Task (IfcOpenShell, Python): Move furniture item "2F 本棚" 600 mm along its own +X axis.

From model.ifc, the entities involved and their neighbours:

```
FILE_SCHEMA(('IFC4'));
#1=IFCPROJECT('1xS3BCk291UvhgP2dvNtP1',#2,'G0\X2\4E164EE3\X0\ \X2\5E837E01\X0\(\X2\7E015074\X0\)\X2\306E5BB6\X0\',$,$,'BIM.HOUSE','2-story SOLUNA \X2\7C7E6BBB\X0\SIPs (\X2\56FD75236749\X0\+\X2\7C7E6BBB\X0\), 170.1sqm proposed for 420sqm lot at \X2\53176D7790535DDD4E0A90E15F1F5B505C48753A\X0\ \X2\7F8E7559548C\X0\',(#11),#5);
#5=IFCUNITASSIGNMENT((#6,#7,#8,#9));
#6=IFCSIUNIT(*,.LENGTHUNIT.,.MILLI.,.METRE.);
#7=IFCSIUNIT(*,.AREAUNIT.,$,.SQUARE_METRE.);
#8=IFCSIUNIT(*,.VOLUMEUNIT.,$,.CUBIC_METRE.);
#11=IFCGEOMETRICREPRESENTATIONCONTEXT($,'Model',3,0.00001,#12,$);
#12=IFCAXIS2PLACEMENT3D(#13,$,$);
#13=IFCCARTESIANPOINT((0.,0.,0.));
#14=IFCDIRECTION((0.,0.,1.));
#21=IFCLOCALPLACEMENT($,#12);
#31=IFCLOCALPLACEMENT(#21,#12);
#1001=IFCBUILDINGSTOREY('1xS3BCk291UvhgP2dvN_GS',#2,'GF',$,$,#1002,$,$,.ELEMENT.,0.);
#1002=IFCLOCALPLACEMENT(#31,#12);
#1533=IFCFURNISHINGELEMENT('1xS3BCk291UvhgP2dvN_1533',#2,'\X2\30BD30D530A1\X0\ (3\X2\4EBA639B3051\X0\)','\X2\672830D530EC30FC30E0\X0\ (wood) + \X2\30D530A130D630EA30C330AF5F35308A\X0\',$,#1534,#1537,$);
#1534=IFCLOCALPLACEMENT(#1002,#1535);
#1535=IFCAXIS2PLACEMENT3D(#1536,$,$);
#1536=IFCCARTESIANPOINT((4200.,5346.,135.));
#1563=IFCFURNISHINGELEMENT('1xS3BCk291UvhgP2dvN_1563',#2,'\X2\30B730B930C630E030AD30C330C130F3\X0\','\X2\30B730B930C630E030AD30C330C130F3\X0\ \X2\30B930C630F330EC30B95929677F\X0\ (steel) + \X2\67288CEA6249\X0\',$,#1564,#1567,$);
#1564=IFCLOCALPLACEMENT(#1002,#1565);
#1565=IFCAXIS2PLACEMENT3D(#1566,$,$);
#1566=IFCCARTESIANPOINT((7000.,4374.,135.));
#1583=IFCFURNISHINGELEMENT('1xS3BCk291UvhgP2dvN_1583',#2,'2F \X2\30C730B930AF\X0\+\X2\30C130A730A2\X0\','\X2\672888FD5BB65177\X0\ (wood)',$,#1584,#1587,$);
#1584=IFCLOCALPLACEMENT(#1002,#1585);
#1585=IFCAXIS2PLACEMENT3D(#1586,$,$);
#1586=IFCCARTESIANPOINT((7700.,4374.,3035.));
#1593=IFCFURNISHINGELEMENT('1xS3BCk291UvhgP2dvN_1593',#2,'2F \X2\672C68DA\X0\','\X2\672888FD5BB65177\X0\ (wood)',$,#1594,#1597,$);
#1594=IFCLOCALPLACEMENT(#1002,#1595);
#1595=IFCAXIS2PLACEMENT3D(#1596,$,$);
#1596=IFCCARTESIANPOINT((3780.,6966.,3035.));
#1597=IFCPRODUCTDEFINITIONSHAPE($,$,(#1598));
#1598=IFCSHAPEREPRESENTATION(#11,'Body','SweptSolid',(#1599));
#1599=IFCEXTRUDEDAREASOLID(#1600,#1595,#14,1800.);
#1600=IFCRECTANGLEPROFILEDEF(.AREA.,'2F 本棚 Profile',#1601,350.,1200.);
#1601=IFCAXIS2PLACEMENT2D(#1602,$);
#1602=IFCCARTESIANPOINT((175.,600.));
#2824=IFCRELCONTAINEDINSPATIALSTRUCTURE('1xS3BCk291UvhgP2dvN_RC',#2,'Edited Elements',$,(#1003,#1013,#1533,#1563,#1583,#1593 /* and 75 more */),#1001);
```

```python
import ifcopenshell
import ifcopenshell.api.geometry
import ifcopenshell.util.placement
import ifcopenshell.util.unit

model = ifcopenshell.open("model.ifc")
unit_scale = ifcopenshell.util.unit.calculate_unit_scale(model)

item = model.by_id(1593)
matrix = ifcopenshell.util.placement.get_local_placement(item.ObjectPlacement)
matrix[:3, 3] += matrix[:3, 0] * 0.6 / unit_scale
ifcopenshell.api.geometry.edit_object_placement(model, product=item, matrix=matrix, is_si=False)

print(ifcopenshell.util.placement.get_local_placement(item.ObjectPlacement).round(3) + 0.0)

model.write("model_rev.ifc")
```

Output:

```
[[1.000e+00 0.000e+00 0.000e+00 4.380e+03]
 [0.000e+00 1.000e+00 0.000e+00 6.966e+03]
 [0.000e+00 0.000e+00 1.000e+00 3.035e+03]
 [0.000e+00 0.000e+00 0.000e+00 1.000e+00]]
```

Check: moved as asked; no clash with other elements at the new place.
